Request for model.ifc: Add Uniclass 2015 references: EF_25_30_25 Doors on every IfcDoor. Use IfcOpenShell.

First a look at what the model holds.

```python
import ifcopenshell

model = ifcopenshell.open("model.ifc")
print(model.schema)
print("classifications:", [c.Name for c in model.by_type("IfcClassification")])
for ifc_class in ("IfcDoor", "IfcRoof", "IfcStair", "IfcWall", "IfcWindow"):
    print(ifc_class, len(model.by_type(ifc_class)))
```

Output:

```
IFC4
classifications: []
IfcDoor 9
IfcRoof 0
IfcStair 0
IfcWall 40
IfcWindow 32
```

```python
import ifcopenshell
import ifcopenshell.api.classification

model = ifcopenshell.open("model.ifc")

system = ifcopenshell.api.classification.add_classification(model, classification="Uniclass 2015")

codes = {
    "IfcDoor": ("EF_25_30_25", "Doors"),
}
for ifc_class, (code, name) in codes.items():
    products = model.by_type(ifc_class)
    ifcopenshell.api.classification.add_reference(
        model, products=products, classification=system, identification=code, name=name
    )
    print(code, len(products))

model.write("model_edited.ifc")
```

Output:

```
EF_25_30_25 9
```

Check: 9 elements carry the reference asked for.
